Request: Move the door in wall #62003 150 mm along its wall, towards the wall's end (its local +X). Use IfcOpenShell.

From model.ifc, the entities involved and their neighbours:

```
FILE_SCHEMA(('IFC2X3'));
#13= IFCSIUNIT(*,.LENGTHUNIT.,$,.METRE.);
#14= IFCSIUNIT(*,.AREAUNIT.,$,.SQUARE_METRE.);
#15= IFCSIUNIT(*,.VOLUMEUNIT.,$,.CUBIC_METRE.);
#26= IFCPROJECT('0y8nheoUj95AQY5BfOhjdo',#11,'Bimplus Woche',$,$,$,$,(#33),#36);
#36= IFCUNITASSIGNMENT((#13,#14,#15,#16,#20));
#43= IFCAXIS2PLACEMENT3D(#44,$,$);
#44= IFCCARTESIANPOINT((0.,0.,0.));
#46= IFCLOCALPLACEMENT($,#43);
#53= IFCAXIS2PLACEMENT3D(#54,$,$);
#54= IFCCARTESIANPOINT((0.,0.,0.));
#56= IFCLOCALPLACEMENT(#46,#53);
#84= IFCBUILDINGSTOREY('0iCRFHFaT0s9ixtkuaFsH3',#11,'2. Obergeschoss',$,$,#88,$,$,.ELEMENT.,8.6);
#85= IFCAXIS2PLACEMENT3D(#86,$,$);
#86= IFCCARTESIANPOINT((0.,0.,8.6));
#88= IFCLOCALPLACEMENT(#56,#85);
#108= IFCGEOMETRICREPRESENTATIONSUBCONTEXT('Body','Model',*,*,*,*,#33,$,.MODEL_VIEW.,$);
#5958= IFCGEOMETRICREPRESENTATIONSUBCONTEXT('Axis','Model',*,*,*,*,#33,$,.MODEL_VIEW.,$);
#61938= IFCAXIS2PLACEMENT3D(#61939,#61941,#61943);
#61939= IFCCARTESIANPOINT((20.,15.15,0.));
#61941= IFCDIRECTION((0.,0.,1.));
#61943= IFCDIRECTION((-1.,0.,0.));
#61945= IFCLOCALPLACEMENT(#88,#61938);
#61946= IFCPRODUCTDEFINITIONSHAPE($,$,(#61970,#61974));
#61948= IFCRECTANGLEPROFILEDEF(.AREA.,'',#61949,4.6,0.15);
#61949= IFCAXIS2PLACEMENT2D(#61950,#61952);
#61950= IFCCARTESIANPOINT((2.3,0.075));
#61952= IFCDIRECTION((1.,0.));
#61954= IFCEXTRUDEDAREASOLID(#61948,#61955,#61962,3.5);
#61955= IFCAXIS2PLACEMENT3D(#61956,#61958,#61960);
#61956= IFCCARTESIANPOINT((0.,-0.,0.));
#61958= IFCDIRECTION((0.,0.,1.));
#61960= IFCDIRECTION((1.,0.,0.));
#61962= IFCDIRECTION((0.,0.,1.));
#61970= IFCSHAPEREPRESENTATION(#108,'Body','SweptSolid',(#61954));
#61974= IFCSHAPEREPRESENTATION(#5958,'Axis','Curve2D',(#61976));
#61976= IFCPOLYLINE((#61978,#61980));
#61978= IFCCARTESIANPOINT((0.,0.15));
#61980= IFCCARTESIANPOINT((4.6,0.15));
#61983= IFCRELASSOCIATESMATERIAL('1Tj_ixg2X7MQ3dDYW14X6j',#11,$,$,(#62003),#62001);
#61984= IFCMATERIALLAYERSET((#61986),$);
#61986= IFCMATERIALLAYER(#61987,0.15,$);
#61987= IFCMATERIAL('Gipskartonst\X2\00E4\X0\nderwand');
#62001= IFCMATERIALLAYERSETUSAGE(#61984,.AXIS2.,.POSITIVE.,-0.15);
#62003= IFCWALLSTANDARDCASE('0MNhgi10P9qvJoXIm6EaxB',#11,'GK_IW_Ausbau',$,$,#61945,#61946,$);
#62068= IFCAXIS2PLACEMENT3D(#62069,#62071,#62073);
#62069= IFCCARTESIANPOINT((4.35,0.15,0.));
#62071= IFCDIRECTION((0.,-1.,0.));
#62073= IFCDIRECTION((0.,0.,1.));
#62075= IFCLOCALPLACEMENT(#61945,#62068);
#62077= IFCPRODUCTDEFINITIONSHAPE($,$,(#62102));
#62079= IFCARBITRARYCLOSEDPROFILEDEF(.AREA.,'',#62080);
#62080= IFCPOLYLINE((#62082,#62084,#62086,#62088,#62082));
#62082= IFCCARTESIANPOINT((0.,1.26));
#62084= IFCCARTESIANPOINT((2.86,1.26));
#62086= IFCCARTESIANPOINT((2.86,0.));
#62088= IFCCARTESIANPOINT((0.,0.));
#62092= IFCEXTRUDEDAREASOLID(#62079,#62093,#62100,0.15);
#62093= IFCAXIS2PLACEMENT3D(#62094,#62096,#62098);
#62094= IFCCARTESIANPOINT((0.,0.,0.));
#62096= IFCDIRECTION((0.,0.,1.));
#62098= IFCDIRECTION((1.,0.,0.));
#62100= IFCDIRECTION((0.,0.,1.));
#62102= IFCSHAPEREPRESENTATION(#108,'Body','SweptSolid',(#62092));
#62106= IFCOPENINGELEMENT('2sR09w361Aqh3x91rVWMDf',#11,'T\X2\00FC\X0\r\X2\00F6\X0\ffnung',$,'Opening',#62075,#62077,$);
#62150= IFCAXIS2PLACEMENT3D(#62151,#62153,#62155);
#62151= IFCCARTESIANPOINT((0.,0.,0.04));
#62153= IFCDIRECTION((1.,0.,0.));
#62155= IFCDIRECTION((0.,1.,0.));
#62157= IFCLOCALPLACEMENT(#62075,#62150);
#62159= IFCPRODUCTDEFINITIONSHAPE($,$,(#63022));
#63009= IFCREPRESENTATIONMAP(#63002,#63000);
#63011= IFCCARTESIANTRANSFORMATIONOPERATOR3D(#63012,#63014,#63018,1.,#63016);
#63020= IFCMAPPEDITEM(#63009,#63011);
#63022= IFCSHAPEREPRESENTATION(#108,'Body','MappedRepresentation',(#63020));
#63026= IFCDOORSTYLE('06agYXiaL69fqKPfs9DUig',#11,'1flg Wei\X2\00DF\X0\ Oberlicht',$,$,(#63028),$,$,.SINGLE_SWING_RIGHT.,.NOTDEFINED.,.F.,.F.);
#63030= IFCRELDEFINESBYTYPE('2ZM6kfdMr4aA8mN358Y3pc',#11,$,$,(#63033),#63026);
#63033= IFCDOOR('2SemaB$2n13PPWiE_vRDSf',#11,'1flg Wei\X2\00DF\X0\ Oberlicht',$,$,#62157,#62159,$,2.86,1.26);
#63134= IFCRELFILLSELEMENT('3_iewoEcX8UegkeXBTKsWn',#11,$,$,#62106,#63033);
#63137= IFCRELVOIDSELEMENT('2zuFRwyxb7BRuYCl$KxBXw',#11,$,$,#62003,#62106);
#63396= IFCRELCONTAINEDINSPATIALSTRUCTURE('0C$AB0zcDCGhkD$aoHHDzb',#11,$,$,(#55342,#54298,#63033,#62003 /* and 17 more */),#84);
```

```python
import ifcopenshell
import ifcopenshell.api.geometry
import ifcopenshell.util.placement

model = ifcopenshell.open("model.ifc")

door = model.by_guid("2SemaB$2n13PPWiE_vRDSf")
opening = door.FillsVoids[0].RelatingOpeningElement
wall = opening.VoidsElements[0].RelatingBuildingElement

wall_matrix = ifcopenshell.util.placement.get_local_placement(wall.ObjectPlacement)
shift = wall_matrix[:3, 0] * 0.15
before = ifcopenshell.util.placement.get_local_placement(door.ObjectPlacement)[:3, 3].copy()

# The door is placed relative to its opening, so it follows when the opening moves.
matrix = ifcopenshell.util.placement.get_local_placement(opening.ObjectPlacement)
matrix[:3, 3] += shift
ifcopenshell.api.geometry.edit_object_placement(
    model, product=opening, matrix=matrix, is_si=False, should_transform_children=True
)

after = ifcopenshell.util.placement.get_local_placement(door.ObjectPlacement)[:3, 3]
print("door moved by", (after - before).round(3) + 0.0)

model.write("model_rev.ifc")
```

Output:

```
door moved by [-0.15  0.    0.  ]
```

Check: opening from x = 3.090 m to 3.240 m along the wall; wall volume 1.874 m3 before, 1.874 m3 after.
